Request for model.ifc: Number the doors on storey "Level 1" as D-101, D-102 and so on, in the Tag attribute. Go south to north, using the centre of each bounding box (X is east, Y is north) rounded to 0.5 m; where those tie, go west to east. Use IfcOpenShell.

First a look at what the model holds.

```python
import ifcopenshell
import ifcopenshell.util.element
import ifcopenshell.util.placement

model = ifcopenshell.open("model.ifc")
print(model.schema)
storey = next(s for s in model.by_type("IfcBuildingStorey") if s.Name == "Level 1")
doors = [e for e in ifcopenshell.util.element.get_decomposition(storey) if e.is_a("IfcDoor")]
for e in sorted(doors, key=lambda e: e.id()):
    origin = ifcopenshell.util.placement.get_local_placement(e.ObjectPlacement)[:3, 3]
    print(e.id(), e.Tag, e.Name, origin.round(2) + 0.0, sep=" | ")
```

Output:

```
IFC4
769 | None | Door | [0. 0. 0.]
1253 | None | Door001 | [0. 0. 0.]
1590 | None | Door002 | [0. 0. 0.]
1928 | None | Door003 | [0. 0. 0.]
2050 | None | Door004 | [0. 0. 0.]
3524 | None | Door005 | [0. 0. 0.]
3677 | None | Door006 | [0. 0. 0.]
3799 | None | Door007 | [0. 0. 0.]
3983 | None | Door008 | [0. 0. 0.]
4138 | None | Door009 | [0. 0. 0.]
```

```python
import ifcopenshell
import ifcopenshell.geom
import ifcopenshell.util.element
import ifcopenshell.util.shape

model = ifcopenshell.open("model.ifc")
settings = ifcopenshell.geom.settings()
settings.set("use-world-coords", True)


def centre(element):
    shape = ifcopenshell.geom.create_shape(settings, element)
    return ifcopenshell.util.shape.get_bbox_centroid(shape.geometry)


storey = next(s for s in model.by_type("IfcBuildingStorey") if s.Name == "Level 1")
doors = [e for e in ifcopenshell.util.element.get_decomposition(storey) if e.is_a("IfcDoor")]

# Insertion points can sit at a corner or the storey origin, so sort by the geometry (in metres).
centres = {e: centre(e) for e in doors}
doors.sort(key=lambda e: (round(centres[e][1] / 0.5), centres[e][0]))

for i, e in enumerate(doors, start=1):
    number = f"D-1{i:02d}"
    e.Tag = number
    print(e.id(), number)

model.write("model_edited.ifc")
```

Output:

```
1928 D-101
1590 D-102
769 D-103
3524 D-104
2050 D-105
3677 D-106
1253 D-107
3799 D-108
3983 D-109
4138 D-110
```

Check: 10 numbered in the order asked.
